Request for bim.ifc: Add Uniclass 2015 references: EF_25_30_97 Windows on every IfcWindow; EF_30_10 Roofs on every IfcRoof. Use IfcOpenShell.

First a look at what the model holds.

```python
import ifcopenshell

model = ifcopenshell.open("bim.ifc")
print(model.schema)
print("classifications:", [c.Name for c in model.by_type("IfcClassification")])
for ifc_class in ("IfcDoor", "IfcRoof", "IfcStair", "IfcWall", "IfcWindow"):
    print(ifc_class, len(model.by_type(ifc_class)))
```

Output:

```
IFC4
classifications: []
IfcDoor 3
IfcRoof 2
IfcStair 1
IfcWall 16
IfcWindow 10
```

```python
import ifcopenshell
import ifcopenshell.api.classification

model = ifcopenshell.open("bim.ifc")

system = ifcopenshell.api.classification.add_classification(model, classification="Uniclass 2015")

codes = {
    "IfcWindow": ("EF_25_30_97", "Windows"),
    "IfcRoof": ("EF_30_10", "Roofs"),
}
for ifc_class, (code, name) in codes.items():
    products = model.by_type(ifc_class)
    ifcopenshell.api.classification.add_reference(
        model, products=products, classification=system, identification=code, name=name
    )
    print(code, len(products))

model.write("bim-out.ifc")
```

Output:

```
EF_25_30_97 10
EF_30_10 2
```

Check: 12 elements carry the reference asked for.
